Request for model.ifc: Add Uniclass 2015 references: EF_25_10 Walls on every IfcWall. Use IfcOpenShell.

First a look at what the model holds.

```python
import ifcopenshell

model = ifcopenshell.open("model.ifc")
print(model.schema)
print("classifications:", [c.Name for c in model.by_type("IfcClassification")])
for ifc_class in ("IfcDoor", "IfcRoof", "IfcStair", "IfcWall", "IfcWindow"):
    print(ifc_class, len(model.by_type(ifc_class)))
```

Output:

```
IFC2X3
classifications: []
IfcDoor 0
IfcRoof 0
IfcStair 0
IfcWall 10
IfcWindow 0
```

```python
import ifcopenshell
import ifcopenshell.api.classification

model = ifcopenshell.open("model.ifc")

# IFC2X3 requires Source and Edition and has no link from the project to the system.
system = model.create_entity("IfcClassification", Source="NBS", Edition="2015", Name="Uniclass 2015")

codes = {
    "IfcWall": ("EF_25_10", "Walls"),
}
for ifc_class, (code, name) in codes.items():
    products = model.by_type(ifc_class)
    ifcopenshell.api.classification.add_reference(
        model, products=products, classification=system, identification=code, name=name
    )
    print(code, len(products))

model.write("model_edited.ifc")
```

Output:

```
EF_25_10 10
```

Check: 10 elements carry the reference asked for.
